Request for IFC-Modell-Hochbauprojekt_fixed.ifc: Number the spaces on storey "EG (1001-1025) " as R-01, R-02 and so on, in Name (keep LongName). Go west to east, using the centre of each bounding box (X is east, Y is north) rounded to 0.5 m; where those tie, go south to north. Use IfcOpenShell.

First a look at what the model holds.

```python
import ifcopenshell
import ifcopenshell.util.element
import ifcopenshell.util.placement

model = ifcopenshell.open("IFC-Modell-Hochbauprojekt_fixed.ifc")
print(model.schema)
storey = next(s for s in model.by_type("IfcBuildingStorey") if s.Name == "EG (1001-1025) ")
spaces = [e for e in ifcopenshell.util.element.get_decomposition(storey) if e.is_a("IfcSpace")]
for e in sorted(spaces, key=lambda e: e.id()):
    origin = ifcopenshell.util.placement.get_local_placement(e.ObjectPlacement)[:3, 3]
    print(e.id(), e.Name, e.LongName, origin.round(2) + 0.0, sep=" | ")
```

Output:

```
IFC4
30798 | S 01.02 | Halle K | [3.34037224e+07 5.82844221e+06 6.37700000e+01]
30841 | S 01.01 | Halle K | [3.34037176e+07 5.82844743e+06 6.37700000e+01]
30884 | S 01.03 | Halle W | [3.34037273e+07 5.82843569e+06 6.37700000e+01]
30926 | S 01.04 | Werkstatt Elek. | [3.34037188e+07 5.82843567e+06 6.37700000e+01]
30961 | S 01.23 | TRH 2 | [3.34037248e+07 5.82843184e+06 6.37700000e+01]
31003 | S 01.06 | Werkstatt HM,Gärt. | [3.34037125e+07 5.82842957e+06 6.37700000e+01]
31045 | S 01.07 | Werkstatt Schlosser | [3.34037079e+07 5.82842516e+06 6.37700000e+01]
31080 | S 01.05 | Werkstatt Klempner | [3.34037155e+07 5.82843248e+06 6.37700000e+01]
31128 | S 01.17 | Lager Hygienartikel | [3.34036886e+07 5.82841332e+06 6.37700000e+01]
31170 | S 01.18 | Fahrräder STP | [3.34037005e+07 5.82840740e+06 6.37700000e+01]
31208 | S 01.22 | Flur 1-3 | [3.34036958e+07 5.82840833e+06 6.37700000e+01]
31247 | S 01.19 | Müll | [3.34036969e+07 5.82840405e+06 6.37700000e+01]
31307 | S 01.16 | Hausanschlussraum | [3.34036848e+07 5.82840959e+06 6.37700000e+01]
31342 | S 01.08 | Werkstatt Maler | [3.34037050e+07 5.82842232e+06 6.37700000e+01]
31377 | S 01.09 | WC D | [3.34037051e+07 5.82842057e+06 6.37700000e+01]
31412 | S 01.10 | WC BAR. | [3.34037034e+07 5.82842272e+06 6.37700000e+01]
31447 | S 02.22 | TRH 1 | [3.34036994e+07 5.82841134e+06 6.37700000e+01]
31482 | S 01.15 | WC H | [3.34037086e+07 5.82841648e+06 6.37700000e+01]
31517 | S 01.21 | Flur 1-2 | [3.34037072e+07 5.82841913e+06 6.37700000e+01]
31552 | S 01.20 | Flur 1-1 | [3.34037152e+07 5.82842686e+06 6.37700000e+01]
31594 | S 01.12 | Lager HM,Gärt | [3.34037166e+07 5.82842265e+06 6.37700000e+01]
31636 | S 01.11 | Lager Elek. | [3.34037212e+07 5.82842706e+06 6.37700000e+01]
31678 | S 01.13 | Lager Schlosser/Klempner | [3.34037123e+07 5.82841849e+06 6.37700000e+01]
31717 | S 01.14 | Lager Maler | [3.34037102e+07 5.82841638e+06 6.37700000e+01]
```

```python
import ifcopenshell
import ifcopenshell.geom
import ifcopenshell.util.element
import ifcopenshell.util.shape

model = ifcopenshell.open("IFC-Modell-Hochbauprojekt_fixed.ifc")
settings = ifcopenshell.geom.settings()
settings.set("use-world-coords", True)


def centre(element):
    shape = ifcopenshell.geom.create_shape(settings, element)
    return ifcopenshell.util.shape.get_bbox_centroid(shape.geometry)


storey = next(s for s in model.by_type("IfcBuildingStorey") if s.Name == "EG (1001-1025) ")
spaces = [e for e in ifcopenshell.util.element.get_decomposition(storey) if e.is_a("IfcSpace")]

# Insertion points can sit at a corner or the storey origin, so sort by the geometry (in metres).
centres = {e: centre(e) for e in spaces}
spaces.sort(key=lambda e: (round(centres[e][0] / 0.5), centres[e][1]))

for i, e in enumerate(spaces, start=1):
    number = f"R-{i:02d}"
    e.Name = number
    print(e.id(), number)

model.write("IFC-Modell-Hochbauprojekt_fixed_edited.ifc")
```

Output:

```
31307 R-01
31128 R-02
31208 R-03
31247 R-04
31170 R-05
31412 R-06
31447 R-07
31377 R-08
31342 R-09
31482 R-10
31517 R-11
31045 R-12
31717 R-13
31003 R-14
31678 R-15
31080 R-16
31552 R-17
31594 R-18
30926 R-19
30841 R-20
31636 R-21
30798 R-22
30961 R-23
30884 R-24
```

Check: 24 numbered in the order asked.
